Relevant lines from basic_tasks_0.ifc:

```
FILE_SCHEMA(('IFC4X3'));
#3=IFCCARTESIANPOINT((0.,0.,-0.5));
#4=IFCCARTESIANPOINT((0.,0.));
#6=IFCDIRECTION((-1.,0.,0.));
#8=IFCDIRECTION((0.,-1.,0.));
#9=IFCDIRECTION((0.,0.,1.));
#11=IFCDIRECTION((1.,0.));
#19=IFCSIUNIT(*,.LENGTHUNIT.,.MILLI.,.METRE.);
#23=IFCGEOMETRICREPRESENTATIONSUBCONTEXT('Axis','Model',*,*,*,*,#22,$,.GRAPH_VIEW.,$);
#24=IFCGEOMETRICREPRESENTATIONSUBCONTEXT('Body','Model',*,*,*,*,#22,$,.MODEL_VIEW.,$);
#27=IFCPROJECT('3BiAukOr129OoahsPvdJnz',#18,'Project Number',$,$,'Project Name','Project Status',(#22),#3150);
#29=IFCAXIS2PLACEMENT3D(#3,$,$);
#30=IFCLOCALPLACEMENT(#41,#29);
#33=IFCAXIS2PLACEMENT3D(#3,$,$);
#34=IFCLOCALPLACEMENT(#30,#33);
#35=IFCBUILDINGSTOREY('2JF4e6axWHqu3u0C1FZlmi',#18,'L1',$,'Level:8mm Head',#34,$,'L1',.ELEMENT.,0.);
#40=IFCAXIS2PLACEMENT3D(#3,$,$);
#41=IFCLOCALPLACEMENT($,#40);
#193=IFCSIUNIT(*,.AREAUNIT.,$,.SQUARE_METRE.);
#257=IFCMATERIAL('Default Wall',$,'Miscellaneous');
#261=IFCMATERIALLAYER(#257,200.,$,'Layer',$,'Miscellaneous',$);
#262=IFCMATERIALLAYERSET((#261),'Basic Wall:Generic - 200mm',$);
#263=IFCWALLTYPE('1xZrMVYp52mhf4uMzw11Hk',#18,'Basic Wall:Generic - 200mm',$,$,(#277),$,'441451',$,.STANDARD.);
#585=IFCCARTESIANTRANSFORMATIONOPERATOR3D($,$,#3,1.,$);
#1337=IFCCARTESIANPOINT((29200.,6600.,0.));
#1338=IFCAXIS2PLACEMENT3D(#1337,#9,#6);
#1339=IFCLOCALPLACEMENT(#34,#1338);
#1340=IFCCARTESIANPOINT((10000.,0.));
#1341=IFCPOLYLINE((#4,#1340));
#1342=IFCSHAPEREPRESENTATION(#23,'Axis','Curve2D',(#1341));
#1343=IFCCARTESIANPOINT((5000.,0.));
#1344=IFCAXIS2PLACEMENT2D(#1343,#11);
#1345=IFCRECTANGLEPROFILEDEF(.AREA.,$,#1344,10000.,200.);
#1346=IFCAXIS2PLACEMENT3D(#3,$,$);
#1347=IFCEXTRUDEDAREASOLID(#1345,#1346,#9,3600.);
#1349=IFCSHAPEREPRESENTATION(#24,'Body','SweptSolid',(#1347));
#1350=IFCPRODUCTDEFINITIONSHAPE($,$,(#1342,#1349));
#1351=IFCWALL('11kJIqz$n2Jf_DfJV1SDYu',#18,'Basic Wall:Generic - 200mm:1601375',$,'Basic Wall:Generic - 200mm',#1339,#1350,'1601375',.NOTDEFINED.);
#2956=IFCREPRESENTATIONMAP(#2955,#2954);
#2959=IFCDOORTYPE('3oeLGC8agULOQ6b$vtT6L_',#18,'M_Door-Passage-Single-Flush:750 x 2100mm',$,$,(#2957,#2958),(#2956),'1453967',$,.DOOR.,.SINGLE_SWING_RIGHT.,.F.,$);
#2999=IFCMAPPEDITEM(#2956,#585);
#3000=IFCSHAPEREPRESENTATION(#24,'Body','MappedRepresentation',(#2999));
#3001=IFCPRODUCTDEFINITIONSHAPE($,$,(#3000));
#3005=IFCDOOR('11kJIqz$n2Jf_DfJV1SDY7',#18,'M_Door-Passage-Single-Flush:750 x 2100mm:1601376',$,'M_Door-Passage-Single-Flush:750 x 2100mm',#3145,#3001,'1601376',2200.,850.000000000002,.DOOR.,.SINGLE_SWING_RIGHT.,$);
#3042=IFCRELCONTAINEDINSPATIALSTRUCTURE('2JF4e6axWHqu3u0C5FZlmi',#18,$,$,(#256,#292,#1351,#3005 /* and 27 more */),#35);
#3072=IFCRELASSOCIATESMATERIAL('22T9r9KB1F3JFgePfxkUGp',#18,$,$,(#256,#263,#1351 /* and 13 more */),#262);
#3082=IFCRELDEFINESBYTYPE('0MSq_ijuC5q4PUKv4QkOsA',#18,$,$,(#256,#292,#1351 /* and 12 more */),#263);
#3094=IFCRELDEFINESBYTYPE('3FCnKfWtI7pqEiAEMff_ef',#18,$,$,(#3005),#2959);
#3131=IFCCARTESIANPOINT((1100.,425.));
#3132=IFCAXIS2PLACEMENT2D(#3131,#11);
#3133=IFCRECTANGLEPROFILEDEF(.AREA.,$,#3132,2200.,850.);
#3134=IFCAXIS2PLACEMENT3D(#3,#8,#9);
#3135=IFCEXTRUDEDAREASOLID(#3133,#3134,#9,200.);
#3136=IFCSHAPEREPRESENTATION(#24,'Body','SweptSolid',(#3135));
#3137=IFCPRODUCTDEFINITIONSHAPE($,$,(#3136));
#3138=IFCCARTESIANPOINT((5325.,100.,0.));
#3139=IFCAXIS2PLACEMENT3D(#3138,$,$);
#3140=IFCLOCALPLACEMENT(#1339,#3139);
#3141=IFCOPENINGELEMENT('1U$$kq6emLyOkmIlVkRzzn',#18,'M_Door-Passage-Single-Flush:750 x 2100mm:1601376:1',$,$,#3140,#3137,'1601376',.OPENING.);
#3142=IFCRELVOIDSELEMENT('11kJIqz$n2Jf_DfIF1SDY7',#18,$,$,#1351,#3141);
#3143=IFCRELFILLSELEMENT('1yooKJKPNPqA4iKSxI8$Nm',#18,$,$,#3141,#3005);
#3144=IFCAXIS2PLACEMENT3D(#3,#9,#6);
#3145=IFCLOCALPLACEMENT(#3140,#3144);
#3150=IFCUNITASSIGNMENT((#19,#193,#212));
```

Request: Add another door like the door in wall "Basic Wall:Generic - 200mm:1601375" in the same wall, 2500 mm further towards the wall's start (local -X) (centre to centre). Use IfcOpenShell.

```python
import ifcopenshell
import ifcopenshell.api.feature
import ifcopenshell.api.geometry
import ifcopenshell.api.root
import ifcopenshell.geom
import ifcopenshell.util.element
import ifcopenshell.util.placement
import ifcopenshell.util.shape
import ifcopenshell.util.unit

model = ifcopenshell.open("basic_tasks_0.ifc")
unit_scale = ifcopenshell.util.unit.calculate_unit_scale(model)
settings = ifcopenshell.geom.settings()


def volume(element):
    """Net volume in cubic metres, openings subtracted."""
    shape = ifcopenshell.geom.create_shape(settings, element)
    return ifcopenshell.util.shape.get_volume(shape.geometry)


def reuse_history(source, copy):
    """copy_class also copies each property set's owner history, people and application; keep the originals."""
    for rel in copy.IsDefinedBy:
        if rel.is_a("IfcRelDefinesByProperties") and (history := rel.RelatingPropertyDefinition.OwnerHistory):
            rel.RelatingPropertyDefinition.OwnerHistory = source.OwnerHistory
            ifcopenshell.util.element.remove_deep2(model, history)


door = model.by_guid("11kJIqz$n2Jf_DfJV1SDY7")
opening = door.FillsVoids[0].RelatingOpeningElement
wall = opening.VoidsElements[0].RelatingBuildingElement
before = volume(wall)
shift = ifcopenshell.util.placement.get_local_placement(wall.ObjectPlacement)[:3, 0] * -2.5 / unit_scale

# copy_class copies the void relationship, type, container and properties, but no geometry.
new_opening = ifcopenshell.api.root.copy_class(model, product=opening)
new_opening.Representation = ifcopenshell.util.element.copy_deep(
    model, opening.Representation, exclude=["IfcGeometricRepresentationContext", "IfcRepresentationMap"]
)
new_opening.Name = "M_Door-Passage-Single-Flush:750 x 2100mm"
new_opening.Tag = None
new_door = ifcopenshell.api.root.copy_class(model, product=door)
new_door.Representation = ifcopenshell.util.element.copy_deep(
    model, door.Representation, exclude=["IfcGeometricRepresentationContext", "IfcRepresentationMap"]
)
new_door.Name = "M_Door-Passage-Single-Flush:750 x 2100mm"
new_door.Tag = None
reuse_history(door, new_door)
ifcopenshell.api.feature.add_filling(model, opening=new_opening, element=new_door)

for old, new in ((opening, new_opening), (door, new_door)):
    matrix = ifcopenshell.util.placement.get_local_placement(old.ObjectPlacement)
    matrix[:3, 3] += shift
    ifcopenshell.api.geometry.edit_object_placement(model, product=new, matrix=matrix, is_si=False)

after = volume(wall)

print(f"wall volume {before:.3f} -> {after:.3f} m3")

model.write("basic_tasks_0_edited.ifc")
```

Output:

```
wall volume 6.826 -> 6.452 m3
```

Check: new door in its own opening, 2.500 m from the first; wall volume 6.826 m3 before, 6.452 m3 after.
